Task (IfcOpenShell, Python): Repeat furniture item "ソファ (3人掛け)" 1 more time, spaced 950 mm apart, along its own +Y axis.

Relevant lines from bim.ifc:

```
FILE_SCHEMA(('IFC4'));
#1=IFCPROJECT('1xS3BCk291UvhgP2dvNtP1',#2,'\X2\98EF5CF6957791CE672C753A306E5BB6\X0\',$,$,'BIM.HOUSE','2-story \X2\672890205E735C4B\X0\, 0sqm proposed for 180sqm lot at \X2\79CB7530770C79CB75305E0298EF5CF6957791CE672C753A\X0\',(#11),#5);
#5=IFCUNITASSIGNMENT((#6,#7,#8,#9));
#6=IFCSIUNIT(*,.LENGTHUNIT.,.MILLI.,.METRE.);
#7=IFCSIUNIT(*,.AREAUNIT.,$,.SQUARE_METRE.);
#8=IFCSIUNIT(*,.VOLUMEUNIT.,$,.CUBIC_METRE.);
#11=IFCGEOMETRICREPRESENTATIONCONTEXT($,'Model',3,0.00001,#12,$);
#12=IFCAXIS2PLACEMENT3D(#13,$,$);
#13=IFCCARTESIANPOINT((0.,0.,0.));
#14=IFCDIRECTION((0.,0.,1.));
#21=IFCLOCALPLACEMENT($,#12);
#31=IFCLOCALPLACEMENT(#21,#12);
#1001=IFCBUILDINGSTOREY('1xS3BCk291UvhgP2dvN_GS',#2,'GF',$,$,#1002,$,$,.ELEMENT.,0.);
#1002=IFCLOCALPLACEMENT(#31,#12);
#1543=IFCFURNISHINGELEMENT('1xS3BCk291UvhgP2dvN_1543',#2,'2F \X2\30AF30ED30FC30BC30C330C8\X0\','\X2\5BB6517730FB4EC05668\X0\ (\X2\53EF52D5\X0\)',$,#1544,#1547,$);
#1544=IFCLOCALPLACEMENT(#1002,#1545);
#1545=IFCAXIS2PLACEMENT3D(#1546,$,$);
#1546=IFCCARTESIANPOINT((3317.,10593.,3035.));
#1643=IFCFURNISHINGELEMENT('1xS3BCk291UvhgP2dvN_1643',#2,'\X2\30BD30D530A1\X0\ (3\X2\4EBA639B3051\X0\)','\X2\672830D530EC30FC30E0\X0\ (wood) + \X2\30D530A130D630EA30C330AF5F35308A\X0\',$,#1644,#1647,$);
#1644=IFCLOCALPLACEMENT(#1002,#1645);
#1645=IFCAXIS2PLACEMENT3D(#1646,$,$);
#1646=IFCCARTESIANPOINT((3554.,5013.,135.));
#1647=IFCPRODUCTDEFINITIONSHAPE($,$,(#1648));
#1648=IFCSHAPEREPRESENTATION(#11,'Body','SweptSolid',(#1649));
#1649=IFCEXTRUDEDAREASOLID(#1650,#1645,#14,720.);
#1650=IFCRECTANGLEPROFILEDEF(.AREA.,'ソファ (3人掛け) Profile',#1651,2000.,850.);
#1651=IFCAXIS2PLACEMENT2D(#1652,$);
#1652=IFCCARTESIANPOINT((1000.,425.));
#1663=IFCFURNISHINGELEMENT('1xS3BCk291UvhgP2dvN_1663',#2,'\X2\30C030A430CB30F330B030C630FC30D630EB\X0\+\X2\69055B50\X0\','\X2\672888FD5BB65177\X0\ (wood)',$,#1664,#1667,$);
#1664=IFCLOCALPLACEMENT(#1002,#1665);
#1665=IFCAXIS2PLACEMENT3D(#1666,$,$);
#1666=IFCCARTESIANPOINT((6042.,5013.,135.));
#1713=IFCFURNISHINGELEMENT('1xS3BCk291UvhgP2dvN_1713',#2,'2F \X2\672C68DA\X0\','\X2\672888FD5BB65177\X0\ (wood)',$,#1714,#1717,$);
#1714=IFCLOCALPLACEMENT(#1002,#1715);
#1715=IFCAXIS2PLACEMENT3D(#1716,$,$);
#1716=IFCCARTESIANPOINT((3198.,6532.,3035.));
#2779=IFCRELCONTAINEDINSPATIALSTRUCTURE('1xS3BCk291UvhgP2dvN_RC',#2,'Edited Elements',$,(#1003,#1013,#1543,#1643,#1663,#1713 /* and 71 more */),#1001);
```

```python
import ifcopenshell
import ifcopenshell.api.geometry
import ifcopenshell.api.root
import ifcopenshell.util.element
import ifcopenshell.util.placement
import ifcopenshell.util.unit

model = ifcopenshell.open("bim.ifc")
unit_scale = ifcopenshell.util.unit.calculate_unit_scale(model)


def reuse_history(source, copy):
    """copy_class also copies each property set's owner history, people and application; keep the originals."""
    for rel in copy.IsDefinedBy:
        if rel.is_a("IfcRelDefinesByProperties") and (history := rel.RelatingPropertyDefinition.OwnerHistory):
            rel.RelatingPropertyDefinition.OwnerHistory = source.OwnerHistory
            ifcopenshell.util.element.remove_deep2(model, history)


source = model.by_guid("1xS3BCk291UvhgP2dvN_1643")
base = ifcopenshell.util.placement.get_local_placement(source.ObjectPlacement)
step = base[:3, 1] * 0.95 / unit_scale

for i in range(1, 2):
    copy = ifcopenshell.api.root.copy_class(model, product=source)
    copy.Representation = ifcopenshell.util.element.copy_deep(
        model, source.Representation, exclude=["IfcGeometricRepresentationContext", "IfcRepresentationMap"]
    )
    reuse_history(source, copy)
    matrix = base.copy()
    matrix[:3, 3] += i * step
    print("added at", matrix[:3, 3].round(3) + 0.0)
    ifcopenshell.api.geometry.edit_object_placement(model, product=copy, matrix=matrix, is_si=False)

model.write("bim_v2.ifc")
```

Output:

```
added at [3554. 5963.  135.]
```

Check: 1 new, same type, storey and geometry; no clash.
